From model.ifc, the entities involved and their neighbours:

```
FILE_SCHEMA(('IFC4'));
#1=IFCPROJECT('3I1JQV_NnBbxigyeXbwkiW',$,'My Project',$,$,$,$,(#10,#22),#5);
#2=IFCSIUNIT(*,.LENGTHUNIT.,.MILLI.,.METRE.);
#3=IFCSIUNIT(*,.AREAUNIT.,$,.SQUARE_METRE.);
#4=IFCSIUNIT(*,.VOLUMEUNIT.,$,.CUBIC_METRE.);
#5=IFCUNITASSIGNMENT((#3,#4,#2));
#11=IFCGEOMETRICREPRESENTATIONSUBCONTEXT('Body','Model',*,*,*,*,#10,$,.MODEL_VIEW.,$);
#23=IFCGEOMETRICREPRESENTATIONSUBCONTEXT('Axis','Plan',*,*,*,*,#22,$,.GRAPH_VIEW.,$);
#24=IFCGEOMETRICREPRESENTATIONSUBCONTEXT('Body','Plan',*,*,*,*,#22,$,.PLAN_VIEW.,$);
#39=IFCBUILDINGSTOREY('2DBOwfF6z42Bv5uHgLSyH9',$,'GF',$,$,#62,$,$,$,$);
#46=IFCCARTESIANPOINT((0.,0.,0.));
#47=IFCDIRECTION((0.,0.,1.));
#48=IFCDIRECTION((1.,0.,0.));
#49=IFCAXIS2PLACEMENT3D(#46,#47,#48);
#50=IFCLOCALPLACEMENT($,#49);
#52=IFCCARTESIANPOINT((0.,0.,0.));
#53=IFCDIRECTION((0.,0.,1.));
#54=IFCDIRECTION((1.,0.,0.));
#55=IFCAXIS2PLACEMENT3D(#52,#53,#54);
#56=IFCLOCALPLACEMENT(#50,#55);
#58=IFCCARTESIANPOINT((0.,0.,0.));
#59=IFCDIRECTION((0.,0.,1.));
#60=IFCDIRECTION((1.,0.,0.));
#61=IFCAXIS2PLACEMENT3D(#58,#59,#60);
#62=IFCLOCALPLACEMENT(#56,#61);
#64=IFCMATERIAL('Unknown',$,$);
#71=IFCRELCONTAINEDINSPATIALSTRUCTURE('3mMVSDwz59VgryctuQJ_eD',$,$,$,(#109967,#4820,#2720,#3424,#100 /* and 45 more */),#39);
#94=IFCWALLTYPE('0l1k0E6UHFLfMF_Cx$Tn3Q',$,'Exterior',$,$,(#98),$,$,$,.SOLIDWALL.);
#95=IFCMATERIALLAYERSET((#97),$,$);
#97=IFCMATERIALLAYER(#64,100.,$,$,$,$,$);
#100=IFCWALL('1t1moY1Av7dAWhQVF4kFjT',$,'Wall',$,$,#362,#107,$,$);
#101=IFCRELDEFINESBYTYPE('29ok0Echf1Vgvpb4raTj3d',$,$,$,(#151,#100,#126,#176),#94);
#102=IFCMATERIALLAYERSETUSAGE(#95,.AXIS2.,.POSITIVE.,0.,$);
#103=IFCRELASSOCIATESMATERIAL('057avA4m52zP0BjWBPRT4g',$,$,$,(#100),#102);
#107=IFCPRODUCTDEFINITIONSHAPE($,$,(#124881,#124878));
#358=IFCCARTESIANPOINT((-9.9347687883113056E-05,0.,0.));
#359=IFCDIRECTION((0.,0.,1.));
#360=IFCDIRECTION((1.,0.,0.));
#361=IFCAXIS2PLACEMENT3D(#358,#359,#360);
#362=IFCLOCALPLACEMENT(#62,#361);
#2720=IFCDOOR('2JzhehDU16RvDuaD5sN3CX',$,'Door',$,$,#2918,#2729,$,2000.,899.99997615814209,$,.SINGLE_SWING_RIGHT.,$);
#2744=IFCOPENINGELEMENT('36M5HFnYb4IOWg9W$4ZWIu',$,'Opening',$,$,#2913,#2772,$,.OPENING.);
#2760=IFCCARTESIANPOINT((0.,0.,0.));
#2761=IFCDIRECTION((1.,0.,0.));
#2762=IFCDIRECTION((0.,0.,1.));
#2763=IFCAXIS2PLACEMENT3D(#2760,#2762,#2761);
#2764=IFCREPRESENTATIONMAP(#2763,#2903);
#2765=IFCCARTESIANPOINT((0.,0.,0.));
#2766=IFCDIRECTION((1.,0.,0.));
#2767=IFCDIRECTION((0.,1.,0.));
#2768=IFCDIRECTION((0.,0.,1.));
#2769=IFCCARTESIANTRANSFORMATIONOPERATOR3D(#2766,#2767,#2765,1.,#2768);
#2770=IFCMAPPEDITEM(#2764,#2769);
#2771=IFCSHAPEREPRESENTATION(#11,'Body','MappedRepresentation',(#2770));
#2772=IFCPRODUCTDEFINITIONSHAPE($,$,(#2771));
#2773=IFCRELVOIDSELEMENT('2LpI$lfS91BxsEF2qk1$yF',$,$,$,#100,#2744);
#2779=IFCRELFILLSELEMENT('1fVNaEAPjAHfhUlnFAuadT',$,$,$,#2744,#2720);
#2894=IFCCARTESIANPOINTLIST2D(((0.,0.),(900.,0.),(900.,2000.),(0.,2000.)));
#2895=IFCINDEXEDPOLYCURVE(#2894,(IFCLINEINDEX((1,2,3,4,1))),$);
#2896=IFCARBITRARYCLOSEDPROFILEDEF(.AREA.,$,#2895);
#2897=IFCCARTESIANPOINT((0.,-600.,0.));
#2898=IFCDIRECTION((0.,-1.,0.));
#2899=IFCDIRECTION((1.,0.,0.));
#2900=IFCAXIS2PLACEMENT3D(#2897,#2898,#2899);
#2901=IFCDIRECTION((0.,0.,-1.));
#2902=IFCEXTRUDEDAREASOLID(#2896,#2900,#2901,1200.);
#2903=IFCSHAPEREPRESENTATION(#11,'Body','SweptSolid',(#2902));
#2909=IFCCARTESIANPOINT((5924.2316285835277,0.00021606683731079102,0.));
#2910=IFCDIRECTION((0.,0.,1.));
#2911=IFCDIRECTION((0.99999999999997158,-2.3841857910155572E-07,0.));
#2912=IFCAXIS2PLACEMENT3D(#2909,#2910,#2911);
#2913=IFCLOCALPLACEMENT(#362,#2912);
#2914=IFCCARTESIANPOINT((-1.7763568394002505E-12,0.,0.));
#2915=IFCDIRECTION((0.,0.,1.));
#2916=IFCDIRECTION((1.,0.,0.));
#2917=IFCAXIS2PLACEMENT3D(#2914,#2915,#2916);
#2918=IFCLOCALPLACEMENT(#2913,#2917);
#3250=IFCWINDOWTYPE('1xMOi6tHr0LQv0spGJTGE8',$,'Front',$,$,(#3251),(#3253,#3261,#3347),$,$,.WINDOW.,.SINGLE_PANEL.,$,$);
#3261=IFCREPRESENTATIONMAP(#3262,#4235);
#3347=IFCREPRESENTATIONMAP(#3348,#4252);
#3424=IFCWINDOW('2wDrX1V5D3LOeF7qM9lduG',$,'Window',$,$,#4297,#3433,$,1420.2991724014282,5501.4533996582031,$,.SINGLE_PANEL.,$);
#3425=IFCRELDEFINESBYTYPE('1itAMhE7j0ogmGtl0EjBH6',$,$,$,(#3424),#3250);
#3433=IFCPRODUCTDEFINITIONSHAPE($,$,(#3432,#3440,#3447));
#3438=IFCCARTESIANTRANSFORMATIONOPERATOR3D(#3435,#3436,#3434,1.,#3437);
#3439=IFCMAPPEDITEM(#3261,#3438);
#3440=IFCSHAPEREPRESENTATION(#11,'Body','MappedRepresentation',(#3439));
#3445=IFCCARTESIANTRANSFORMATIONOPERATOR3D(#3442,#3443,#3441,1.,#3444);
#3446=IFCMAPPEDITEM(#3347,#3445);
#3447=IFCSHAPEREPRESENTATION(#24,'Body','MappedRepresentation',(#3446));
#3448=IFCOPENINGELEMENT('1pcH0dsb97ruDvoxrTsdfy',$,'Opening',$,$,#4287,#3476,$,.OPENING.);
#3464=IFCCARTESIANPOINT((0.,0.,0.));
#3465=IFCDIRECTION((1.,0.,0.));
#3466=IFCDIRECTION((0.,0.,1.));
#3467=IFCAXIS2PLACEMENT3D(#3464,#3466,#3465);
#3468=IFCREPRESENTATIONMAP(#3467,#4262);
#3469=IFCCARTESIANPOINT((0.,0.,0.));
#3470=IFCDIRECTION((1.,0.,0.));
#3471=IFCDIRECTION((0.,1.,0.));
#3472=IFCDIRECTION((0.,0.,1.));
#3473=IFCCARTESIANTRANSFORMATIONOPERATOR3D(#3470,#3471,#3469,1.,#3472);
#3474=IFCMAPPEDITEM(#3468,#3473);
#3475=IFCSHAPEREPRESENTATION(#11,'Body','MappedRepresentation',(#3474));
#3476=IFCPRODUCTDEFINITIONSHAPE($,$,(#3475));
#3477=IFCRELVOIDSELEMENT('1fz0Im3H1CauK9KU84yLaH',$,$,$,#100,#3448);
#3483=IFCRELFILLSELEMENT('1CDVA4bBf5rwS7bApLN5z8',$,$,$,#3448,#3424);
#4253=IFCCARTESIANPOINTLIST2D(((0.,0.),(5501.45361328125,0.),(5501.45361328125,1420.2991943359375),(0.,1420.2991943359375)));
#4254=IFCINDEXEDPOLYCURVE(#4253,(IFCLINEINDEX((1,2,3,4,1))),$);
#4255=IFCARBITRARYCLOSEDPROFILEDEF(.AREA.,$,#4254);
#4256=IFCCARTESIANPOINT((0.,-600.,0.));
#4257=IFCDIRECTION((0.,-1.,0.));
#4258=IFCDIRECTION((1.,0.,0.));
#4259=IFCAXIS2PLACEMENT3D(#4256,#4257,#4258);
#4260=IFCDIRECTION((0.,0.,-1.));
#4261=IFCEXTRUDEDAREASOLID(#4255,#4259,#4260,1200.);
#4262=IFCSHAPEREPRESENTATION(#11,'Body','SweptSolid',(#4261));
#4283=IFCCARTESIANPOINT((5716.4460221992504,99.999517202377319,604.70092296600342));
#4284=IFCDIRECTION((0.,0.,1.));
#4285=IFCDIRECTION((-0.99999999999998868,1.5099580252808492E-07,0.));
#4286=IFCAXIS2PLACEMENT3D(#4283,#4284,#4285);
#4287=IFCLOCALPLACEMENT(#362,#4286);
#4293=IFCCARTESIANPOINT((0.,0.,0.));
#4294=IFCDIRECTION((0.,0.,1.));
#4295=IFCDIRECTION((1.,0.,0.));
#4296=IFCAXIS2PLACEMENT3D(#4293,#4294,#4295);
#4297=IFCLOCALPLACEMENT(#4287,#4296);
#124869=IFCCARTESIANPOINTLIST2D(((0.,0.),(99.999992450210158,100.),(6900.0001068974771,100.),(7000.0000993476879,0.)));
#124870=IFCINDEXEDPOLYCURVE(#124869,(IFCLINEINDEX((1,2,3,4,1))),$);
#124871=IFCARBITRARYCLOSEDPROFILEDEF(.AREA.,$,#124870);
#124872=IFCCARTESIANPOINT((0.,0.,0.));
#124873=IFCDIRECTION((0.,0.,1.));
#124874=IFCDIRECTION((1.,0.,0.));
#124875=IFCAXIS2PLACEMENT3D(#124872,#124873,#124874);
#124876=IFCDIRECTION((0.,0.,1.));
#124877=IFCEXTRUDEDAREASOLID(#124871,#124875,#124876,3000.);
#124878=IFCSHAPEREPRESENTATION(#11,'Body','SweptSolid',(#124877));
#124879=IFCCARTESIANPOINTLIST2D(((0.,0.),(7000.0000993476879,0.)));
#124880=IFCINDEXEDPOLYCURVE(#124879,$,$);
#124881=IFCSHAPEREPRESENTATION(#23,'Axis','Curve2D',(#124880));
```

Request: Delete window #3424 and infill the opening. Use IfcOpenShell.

```python
import ifcopenshell
import ifcopenshell.api.feature
import ifcopenshell.api.root
import ifcopenshell.geom
import ifcopenshell.util.shape

model = ifcopenshell.open("model.ifc")
settings = ifcopenshell.geom.settings()


def volume(element):
    """Net volume in cubic metres, openings subtracted."""
    shape = ifcopenshell.geom.create_shape(settings, element)
    return ifcopenshell.util.shape.get_volume(shape.geometry)


window = model.by_guid("2wDrX1V5D3LOeF7qM9lduG")
opening = window.FillsVoids[0].RelatingOpeningElement
wall = opening.VoidsElements[0].RelatingBuildingElement
before = volume(wall)

ifcopenshell.api.root.remove_product(model, product=window)
ifcopenshell.api.feature.remove_feature(model, feature=opening)

after = volume(wall)

print(f"wall volume {before:.3f} -> {after:.3f} m3")

model.write("model_updated.ifc")
```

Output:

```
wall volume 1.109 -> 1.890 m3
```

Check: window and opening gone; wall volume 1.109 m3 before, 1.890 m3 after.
